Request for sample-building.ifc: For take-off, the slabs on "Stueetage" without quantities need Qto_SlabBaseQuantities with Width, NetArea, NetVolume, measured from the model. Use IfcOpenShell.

First a look at what the model holds.

```python
import ifcopenshell
import ifcopenshell.util.element
import ifcopenshell.util.unit

model = ifcopenshell.open("sample-building.ifc")
print(model.schema)
for unit_type in ("LENGTHUNIT", "AREAUNIT", "VOLUMEUNIT"):
    print(unit_type, ifcopenshell.util.unit.calculate_unit_scale(model, unit_type))
storey = next(s for s in model.by_type("IfcBuildingStorey") if s.Name == "Stueetage")
slabs = [e for e in ifcopenshell.util.element.get_decomposition(storey) if e.is_a("IfcSlab")]
for e in sorted(slabs, key=lambda e: e.id()):
    print(e.id(), e.is_a(), e.Name, list(ifcopenshell.util.element.get_psets(e, qtos_only=True)), sep=" | ")
```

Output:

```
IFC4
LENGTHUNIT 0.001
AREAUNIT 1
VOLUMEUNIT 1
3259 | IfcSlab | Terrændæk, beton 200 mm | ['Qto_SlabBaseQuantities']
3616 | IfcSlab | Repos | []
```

```python
import ifcopenshell
import ifcopenshell.api.pset
import ifcopenshell.geom
import ifcopenshell.util.element
import ifcopenshell.util.shape
import ifcopenshell.util.unit

model = ifcopenshell.open("sample-building.ifc")
unit_scale = ifcopenshell.util.unit.calculate_unit_scale(model)
area_scale = ifcopenshell.util.unit.calculate_unit_scale(model, "AREAUNIT")
volume_scale = ifcopenshell.util.unit.calculate_unit_scale(model, "VOLUMEUNIT")
settings = ifcopenshell.geom.settings()

storey = next(s for s in model.by_type("IfcBuildingStorey") if s.Name == "Stueetage")
slabs = [e for e in ifcopenshell.util.element.get_decomposition(storey) if e.is_a("IfcSlab")]

for e in sorted(slabs, key=lambda e: e.id()):
    if ifcopenshell.util.element.get_psets(e, qtos_only=True, should_inherit=False):
        continue
    # Geometry comes back in metres, in the element's own axes.
    shape = ifcopenshell.geom.create_shape(settings, e)
    values = {
        "Width": ifcopenshell.util.shape.get_z(shape.geometry) / unit_scale,
        "NetArea": ifcopenshell.util.shape.get_footprint_area(shape.geometry) / area_scale,
        "NetVolume": ifcopenshell.util.shape.get_volume(shape.geometry) / volume_scale,
    }
    qto = ifcopenshell.api.pset.add_qto(model, product=e, name="Qto_SlabBaseQuantities")
    ifcopenshell.api.pset.edit_qto(model, qto=qto, properties=values)
    print(e.id(), {k: round(v, 3) for k, v in values.items()})

model.write("sample-building_updated.ifc")
```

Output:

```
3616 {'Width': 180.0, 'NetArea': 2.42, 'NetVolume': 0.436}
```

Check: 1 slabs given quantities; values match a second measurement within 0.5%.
